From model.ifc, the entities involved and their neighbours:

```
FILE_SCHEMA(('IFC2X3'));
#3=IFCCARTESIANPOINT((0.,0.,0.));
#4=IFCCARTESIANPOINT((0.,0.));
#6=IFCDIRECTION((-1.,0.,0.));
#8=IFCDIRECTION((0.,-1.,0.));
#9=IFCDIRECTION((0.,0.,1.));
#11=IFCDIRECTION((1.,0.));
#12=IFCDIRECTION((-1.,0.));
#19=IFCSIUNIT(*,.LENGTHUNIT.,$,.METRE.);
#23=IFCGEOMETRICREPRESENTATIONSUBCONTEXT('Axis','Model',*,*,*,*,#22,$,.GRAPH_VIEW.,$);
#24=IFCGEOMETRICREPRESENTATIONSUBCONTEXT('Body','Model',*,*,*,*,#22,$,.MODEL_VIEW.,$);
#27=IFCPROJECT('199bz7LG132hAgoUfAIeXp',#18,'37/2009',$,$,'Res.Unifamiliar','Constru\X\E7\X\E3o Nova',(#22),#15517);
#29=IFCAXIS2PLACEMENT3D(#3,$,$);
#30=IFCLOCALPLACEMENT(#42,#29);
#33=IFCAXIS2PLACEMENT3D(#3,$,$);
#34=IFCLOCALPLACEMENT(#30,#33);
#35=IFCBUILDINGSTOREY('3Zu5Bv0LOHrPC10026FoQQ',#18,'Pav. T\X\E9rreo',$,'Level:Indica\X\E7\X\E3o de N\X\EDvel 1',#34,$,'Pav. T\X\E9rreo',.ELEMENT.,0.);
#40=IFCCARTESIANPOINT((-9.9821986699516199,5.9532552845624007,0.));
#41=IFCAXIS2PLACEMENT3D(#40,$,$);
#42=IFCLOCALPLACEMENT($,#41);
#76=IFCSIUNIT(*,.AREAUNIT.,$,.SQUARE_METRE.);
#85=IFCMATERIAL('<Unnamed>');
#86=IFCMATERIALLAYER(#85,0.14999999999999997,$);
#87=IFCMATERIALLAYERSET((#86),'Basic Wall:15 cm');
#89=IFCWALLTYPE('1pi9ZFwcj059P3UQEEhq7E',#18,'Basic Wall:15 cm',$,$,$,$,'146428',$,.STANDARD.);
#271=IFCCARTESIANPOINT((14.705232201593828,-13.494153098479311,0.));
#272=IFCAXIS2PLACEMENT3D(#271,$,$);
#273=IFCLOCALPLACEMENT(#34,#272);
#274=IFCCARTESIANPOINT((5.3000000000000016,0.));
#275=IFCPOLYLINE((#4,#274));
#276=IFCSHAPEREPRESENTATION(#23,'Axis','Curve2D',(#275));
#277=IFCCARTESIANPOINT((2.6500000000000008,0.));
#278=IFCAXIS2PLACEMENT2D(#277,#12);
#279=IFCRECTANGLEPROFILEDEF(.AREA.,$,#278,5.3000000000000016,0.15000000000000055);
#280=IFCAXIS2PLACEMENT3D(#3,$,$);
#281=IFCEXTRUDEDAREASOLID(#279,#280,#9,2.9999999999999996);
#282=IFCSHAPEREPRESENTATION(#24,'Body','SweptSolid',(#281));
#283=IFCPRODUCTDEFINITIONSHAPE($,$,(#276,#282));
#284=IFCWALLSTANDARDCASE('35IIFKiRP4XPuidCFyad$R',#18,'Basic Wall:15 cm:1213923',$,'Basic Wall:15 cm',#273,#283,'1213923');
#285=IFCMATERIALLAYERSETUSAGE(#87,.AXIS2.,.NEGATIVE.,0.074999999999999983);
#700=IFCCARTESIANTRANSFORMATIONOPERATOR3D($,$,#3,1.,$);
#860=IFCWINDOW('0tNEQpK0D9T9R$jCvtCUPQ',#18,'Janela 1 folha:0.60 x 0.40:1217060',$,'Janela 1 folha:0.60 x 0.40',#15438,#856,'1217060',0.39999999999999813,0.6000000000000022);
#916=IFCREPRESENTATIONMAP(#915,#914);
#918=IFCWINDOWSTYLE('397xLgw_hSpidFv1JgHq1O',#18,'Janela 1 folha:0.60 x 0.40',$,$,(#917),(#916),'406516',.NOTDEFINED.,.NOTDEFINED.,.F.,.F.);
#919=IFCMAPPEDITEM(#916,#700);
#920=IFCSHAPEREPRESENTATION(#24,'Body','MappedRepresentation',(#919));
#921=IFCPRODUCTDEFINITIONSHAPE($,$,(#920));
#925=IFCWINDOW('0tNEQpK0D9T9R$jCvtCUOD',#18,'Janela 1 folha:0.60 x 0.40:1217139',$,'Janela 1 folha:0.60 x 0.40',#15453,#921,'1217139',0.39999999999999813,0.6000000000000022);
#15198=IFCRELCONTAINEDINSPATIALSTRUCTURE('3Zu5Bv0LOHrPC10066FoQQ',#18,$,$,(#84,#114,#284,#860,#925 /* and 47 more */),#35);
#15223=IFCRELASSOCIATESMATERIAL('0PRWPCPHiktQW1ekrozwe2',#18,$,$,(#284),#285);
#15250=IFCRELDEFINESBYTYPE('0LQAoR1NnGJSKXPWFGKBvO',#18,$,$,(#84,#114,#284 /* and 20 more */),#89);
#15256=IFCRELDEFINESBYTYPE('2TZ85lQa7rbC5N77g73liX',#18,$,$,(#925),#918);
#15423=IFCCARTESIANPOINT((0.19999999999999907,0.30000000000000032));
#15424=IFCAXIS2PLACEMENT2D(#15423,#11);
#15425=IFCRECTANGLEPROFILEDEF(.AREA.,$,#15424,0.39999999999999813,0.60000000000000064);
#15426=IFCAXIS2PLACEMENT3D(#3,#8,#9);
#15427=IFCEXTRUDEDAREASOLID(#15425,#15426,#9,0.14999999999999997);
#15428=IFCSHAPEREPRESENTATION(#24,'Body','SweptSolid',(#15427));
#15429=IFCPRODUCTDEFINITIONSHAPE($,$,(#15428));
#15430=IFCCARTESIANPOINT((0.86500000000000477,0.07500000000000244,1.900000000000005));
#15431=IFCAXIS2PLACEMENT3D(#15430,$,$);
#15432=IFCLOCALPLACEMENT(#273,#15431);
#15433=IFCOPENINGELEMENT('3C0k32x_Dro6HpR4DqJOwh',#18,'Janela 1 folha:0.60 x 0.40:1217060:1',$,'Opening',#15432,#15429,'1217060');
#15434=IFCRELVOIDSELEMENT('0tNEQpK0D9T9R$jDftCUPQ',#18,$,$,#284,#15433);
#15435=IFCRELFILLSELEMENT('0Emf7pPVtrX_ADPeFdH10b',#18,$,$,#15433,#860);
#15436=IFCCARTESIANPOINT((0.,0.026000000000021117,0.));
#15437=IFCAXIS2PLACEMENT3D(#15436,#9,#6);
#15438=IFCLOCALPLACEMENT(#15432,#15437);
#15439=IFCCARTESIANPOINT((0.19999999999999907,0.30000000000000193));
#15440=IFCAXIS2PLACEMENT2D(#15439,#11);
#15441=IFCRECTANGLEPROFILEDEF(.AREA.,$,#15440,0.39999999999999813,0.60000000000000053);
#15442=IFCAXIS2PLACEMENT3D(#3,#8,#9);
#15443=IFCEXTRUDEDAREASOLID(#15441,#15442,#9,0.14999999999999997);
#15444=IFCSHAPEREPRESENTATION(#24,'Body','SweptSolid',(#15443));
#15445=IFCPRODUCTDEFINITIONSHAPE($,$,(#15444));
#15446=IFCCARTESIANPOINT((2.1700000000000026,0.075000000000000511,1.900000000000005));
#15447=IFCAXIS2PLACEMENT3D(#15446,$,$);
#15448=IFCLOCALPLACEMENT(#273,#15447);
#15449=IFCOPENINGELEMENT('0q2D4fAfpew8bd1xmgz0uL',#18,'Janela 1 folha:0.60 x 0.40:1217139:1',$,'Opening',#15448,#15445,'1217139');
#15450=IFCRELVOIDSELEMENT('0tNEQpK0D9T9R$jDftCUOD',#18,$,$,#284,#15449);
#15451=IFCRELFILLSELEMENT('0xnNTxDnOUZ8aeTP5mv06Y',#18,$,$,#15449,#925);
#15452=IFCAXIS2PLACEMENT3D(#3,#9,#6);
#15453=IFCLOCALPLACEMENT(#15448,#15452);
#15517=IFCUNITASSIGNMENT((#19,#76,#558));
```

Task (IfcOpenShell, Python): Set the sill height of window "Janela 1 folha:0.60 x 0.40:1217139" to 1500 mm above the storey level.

```python
import numpy as np
import ifcopenshell
import ifcopenshell.api.geometry
import ifcopenshell.geom
import ifcopenshell.util.element
import ifcopenshell.util.placement
import ifcopenshell.util.shape
import ifcopenshell.util.unit

model = ifcopenshell.open("model.ifc")
unit_scale = ifcopenshell.util.unit.calculate_unit_scale(model)

window = model.by_guid("0tNEQpK0D9T9R$jCvtCUOD")
opening = window.FillsVoids[0].RelatingOpeningElement
storey = ifcopenshell.util.element.get_container(window, ifc_class="IfcBuildingStorey")
level = ifcopenshell.util.placement.get_local_placement(storey.ObjectPlacement)[2, 3]

# The opening's origin need not be at the sill, so measure its lowest point.
shape = ifcopenshell.geom.create_shape(ifcopenshell.geom.settings(), opening)
bottom = ifcopenshell.util.shape.get_shape_bottom_elevation(shape, shape.geometry) / unit_scale
dz = level + 1.5 / unit_scale - bottom

shift = np.array([0.0, 0.0, dz])
# The window is placed relative to its opening, so it follows when the opening moves.
matrix = ifcopenshell.util.placement.get_local_placement(opening.ObjectPlacement)
matrix[:3, 3] += shift
ifcopenshell.api.geometry.edit_object_placement(
    model, product=opening, matrix=matrix, is_si=False, should_transform_children=True
)

print(f"moved by {dz * unit_scale:+.3f} m")

model.write("model_v2.ifc")
```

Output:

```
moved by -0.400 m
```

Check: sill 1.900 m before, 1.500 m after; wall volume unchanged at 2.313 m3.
